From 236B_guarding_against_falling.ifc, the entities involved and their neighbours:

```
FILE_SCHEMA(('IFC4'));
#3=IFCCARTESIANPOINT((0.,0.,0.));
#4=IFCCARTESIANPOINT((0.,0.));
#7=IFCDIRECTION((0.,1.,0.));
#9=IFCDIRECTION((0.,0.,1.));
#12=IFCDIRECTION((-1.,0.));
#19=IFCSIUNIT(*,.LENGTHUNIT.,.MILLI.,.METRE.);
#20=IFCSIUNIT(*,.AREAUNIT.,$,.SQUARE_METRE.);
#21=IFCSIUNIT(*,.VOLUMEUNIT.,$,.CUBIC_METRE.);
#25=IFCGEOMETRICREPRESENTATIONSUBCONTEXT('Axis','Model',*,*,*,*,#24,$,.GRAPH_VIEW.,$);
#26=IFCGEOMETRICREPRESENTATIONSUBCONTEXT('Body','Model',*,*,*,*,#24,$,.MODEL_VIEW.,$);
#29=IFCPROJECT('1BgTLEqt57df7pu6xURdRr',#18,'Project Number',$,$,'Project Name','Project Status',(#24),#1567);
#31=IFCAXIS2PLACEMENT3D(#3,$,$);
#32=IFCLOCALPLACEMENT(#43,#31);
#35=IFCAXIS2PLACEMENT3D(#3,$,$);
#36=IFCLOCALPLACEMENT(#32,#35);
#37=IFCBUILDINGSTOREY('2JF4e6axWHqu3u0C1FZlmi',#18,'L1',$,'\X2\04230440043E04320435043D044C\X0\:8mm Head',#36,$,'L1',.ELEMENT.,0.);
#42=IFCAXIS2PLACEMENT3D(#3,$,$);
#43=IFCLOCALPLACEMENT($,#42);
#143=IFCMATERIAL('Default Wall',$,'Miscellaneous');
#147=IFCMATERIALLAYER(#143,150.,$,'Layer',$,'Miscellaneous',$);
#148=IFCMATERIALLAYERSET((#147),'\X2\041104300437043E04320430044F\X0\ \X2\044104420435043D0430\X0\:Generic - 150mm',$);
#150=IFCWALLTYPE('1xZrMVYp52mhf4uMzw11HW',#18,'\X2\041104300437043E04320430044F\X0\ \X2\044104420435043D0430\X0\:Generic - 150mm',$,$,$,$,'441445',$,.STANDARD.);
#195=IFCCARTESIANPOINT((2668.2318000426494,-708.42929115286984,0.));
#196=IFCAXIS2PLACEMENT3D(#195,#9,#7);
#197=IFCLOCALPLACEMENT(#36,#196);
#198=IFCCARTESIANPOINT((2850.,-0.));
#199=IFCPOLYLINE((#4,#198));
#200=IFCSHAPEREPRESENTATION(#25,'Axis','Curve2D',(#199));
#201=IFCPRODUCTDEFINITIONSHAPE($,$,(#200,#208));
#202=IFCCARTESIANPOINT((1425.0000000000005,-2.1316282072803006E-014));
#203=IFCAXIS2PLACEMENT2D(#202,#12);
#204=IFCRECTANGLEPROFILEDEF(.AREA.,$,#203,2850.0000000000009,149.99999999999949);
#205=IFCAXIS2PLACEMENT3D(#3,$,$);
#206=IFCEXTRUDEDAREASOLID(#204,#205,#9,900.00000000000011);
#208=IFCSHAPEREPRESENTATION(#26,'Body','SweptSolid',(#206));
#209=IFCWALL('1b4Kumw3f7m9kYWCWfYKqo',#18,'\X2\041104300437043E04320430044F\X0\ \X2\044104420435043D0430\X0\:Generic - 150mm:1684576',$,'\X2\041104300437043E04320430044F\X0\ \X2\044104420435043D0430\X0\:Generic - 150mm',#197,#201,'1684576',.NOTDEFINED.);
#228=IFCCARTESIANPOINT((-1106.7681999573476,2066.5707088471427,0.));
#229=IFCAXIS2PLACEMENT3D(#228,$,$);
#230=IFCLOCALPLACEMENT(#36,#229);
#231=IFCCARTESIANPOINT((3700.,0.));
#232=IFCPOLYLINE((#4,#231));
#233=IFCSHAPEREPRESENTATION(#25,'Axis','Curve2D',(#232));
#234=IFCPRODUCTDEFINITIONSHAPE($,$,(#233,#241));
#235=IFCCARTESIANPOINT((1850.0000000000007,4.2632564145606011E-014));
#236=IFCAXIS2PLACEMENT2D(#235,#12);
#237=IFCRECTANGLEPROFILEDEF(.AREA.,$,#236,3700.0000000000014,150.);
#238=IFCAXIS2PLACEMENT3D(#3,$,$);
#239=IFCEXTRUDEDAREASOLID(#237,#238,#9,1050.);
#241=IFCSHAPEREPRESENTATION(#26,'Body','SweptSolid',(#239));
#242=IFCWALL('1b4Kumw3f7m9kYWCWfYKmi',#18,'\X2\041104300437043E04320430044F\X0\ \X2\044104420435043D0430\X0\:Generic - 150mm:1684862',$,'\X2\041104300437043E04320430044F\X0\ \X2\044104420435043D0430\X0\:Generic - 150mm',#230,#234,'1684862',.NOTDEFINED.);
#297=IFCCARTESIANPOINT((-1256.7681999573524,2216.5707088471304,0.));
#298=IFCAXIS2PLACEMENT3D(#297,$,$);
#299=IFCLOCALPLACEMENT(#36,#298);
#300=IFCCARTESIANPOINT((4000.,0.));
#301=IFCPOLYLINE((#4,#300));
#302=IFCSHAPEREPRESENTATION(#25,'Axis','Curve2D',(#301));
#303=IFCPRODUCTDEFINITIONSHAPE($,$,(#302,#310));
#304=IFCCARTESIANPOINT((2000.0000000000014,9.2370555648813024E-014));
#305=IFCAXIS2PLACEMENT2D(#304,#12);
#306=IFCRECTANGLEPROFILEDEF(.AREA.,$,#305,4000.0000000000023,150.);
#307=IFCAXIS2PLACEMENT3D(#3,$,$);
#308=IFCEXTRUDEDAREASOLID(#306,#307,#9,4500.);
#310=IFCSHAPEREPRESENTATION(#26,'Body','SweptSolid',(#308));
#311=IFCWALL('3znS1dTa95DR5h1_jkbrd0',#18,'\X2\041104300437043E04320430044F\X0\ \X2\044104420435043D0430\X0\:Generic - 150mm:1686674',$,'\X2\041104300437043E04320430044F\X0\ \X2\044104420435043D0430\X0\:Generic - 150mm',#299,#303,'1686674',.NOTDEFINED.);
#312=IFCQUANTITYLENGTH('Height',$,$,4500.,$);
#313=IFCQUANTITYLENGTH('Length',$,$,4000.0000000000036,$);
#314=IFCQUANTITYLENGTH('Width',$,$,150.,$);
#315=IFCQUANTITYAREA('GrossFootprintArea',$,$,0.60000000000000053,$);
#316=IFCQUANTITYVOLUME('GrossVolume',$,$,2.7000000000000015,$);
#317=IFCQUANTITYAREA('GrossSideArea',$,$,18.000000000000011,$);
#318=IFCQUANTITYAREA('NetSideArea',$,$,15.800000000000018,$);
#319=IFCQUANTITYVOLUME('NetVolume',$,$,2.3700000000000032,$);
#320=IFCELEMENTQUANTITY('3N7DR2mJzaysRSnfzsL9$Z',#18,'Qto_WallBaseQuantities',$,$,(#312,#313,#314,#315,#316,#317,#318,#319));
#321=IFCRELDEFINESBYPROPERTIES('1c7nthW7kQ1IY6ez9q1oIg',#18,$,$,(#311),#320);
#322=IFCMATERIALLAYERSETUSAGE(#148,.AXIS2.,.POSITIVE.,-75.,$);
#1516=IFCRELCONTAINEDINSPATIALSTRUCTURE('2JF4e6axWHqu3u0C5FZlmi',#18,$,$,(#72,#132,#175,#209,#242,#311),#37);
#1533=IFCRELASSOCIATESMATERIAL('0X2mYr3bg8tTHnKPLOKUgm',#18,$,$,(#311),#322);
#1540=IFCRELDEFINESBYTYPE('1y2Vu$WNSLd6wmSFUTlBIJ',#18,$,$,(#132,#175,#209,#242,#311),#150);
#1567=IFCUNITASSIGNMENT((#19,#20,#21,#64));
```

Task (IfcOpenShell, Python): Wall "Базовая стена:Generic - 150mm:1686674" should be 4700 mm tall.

```python
import ifcopenshell
import ifcopenshell.api.pset
import ifcopenshell.geom
import ifcopenshell.util.element
import ifcopenshell.util.representation
import ifcopenshell.util.shape
import ifcopenshell.util.unit

model = ifcopenshell.open("236B_guarding_against_falling.ifc")
unit_scale = ifcopenshell.util.unit.calculate_unit_scale(model)
area_scale = ifcopenshell.util.unit.calculate_unit_scale(model, "AREAUNIT")
volume_scale = ifcopenshell.util.unit.calculate_unit_scale(model, "VOLUMEUNIT")
settings = ifcopenshell.geom.settings()


def volume(element):
    """Net volume in cubic metres, openings subtracted."""
    shape = ifcopenshell.geom.create_shape(settings, element)
    return ifcopenshell.util.shape.get_volume(shape.geometry)


wall = model.by_guid("3znS1dTa95DR5h1_jkbrd0")
before = volume(wall)

body = ifcopenshell.util.representation.get_representation(wall, "Model", "Body")
solid = body.Items[0]
old_height = solid.Depth
solid.Depth = 4.7 / unit_scale
after = volume(wall)
thickness = 0.15  # wall thickness in metres

# Update the stored height, areas and volumes.
qto = model.by_id(ifcopenshell.util.element.get_pset(wall, "Qto_WallBaseQuantities", should_inherit=False)["id"])
ifcopenshell.api.pset.edit_qto(model, qto=qto, properties={
    "Height": solid.Depth,
    "GrossVolume": ifcopenshell.util.element.get_pset(wall, "Qto_WallBaseQuantities", "GrossVolume") * solid.Depth / old_height,
    "GrossSideArea": ifcopenshell.util.element.get_pset(wall, "Qto_WallBaseQuantities", "GrossSideArea") * solid.Depth / old_height,
    "NetSideArea": after / thickness / area_scale,
    "NetVolume": after / volume_scale,
})

print(f"height {old_height:g} -> {solid.Depth:g}, volume {before:.3f} -> {after:.3f} m3")

model.write("236B_guarding_against_falling_rev.ifc")
```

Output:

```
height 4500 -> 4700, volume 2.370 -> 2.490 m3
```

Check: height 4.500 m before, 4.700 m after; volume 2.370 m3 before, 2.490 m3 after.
